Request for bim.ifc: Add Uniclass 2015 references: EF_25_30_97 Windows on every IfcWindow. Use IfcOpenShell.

First a look at what the model holds.

```python
import ifcopenshell

model = ifcopenshell.open("bim.ifc")
print(model.schema)
print("classifications:", [c.Name for c in model.by_type("IfcClassification")])
for ifc_class in ("IfcDoor", "IfcRoof", "IfcStair", "IfcWall", "IfcWindow"):
    print(ifc_class, len(model.by_type(ifc_class)))
```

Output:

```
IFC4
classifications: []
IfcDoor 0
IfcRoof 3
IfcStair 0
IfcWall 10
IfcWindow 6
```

```python
import ifcopenshell
import ifcopenshell.api.classification

model = ifcopenshell.open("bim.ifc")

system = ifcopenshell.api.classification.add_classification(model, classification="Uniclass 2015")

codes = {
    "IfcWindow": ("EF_25_30_97", "Windows"),
}
for ifc_class, (code, name) in codes.items():
    products = model.by_type(ifc_class)
    ifcopenshell.api.classification.add_reference(
        model, products=products, classification=system, identification=code, name=name
    )
    print(code, len(products))

model.write("bim_edited.ifc")
```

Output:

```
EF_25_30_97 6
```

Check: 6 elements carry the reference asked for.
